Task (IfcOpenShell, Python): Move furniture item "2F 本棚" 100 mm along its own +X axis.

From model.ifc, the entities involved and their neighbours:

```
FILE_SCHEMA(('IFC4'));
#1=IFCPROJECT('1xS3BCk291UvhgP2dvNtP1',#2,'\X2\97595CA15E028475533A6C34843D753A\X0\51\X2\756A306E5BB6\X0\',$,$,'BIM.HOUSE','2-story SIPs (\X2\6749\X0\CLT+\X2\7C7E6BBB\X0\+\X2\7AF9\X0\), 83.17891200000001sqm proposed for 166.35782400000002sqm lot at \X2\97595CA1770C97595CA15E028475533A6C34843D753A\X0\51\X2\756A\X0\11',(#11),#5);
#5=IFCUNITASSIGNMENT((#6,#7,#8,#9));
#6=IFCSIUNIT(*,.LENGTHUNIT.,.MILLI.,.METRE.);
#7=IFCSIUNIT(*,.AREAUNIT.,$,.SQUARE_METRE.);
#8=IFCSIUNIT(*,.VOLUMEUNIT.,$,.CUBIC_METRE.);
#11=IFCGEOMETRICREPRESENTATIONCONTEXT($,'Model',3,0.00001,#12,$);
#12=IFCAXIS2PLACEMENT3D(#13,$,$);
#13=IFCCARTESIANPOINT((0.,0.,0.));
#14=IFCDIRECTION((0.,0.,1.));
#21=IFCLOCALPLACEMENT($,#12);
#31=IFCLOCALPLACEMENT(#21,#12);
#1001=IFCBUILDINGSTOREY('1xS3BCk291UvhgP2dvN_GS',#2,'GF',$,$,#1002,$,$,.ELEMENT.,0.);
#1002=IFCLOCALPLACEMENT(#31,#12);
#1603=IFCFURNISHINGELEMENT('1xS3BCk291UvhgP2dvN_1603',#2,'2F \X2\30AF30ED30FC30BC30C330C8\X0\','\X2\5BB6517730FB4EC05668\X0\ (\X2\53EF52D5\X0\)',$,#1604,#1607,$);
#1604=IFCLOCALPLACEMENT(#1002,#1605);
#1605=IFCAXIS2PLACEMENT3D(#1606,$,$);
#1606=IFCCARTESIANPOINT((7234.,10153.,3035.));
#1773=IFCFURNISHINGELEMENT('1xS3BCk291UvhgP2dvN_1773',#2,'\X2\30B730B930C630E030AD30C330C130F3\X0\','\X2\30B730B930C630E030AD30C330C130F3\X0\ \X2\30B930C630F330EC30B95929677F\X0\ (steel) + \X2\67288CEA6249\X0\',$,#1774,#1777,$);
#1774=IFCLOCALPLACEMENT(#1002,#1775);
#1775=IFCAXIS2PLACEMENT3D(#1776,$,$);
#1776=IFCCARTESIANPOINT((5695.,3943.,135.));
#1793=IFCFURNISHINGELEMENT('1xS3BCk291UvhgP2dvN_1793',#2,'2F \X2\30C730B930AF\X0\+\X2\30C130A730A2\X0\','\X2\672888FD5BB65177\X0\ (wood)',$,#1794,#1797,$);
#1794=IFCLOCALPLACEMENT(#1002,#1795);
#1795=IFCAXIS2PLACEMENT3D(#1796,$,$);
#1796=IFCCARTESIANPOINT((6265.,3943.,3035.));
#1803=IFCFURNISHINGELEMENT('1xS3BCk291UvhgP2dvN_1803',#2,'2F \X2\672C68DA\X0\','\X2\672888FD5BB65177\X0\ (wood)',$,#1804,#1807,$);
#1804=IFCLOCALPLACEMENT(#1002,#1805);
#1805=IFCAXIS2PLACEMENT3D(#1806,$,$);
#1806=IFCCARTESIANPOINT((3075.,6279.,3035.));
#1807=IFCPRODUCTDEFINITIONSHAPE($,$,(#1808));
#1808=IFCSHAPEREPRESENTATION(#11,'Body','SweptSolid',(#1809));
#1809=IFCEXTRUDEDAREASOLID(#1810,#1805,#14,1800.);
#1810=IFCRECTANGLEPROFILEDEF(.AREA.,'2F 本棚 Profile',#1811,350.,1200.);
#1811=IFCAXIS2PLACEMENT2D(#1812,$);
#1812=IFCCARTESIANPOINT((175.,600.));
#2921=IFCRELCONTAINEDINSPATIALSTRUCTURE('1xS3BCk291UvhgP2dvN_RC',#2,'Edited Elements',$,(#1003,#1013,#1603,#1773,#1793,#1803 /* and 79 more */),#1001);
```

```python
import ifcopenshell
import ifcopenshell.api.geometry
import ifcopenshell.util.placement

model = ifcopenshell.open("model.ifc")

item = model.by_guid("1xS3BCk291UvhgP2dvN_1803")
matrix = ifcopenshell.util.placement.get_local_placement(item.ObjectPlacement)
matrix[:3, 3] += matrix[:3, 0] * 100.0
ifcopenshell.api.geometry.edit_object_placement(model, product=item, matrix=matrix, is_si=False)

print(ifcopenshell.util.placement.get_local_placement(item.ObjectPlacement).round(3) + 0.0)

model.write("model_edited.ifc")
```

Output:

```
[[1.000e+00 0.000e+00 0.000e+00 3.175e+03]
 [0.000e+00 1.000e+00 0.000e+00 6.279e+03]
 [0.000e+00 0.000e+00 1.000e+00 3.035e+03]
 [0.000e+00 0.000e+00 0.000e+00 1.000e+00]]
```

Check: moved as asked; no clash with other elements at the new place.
